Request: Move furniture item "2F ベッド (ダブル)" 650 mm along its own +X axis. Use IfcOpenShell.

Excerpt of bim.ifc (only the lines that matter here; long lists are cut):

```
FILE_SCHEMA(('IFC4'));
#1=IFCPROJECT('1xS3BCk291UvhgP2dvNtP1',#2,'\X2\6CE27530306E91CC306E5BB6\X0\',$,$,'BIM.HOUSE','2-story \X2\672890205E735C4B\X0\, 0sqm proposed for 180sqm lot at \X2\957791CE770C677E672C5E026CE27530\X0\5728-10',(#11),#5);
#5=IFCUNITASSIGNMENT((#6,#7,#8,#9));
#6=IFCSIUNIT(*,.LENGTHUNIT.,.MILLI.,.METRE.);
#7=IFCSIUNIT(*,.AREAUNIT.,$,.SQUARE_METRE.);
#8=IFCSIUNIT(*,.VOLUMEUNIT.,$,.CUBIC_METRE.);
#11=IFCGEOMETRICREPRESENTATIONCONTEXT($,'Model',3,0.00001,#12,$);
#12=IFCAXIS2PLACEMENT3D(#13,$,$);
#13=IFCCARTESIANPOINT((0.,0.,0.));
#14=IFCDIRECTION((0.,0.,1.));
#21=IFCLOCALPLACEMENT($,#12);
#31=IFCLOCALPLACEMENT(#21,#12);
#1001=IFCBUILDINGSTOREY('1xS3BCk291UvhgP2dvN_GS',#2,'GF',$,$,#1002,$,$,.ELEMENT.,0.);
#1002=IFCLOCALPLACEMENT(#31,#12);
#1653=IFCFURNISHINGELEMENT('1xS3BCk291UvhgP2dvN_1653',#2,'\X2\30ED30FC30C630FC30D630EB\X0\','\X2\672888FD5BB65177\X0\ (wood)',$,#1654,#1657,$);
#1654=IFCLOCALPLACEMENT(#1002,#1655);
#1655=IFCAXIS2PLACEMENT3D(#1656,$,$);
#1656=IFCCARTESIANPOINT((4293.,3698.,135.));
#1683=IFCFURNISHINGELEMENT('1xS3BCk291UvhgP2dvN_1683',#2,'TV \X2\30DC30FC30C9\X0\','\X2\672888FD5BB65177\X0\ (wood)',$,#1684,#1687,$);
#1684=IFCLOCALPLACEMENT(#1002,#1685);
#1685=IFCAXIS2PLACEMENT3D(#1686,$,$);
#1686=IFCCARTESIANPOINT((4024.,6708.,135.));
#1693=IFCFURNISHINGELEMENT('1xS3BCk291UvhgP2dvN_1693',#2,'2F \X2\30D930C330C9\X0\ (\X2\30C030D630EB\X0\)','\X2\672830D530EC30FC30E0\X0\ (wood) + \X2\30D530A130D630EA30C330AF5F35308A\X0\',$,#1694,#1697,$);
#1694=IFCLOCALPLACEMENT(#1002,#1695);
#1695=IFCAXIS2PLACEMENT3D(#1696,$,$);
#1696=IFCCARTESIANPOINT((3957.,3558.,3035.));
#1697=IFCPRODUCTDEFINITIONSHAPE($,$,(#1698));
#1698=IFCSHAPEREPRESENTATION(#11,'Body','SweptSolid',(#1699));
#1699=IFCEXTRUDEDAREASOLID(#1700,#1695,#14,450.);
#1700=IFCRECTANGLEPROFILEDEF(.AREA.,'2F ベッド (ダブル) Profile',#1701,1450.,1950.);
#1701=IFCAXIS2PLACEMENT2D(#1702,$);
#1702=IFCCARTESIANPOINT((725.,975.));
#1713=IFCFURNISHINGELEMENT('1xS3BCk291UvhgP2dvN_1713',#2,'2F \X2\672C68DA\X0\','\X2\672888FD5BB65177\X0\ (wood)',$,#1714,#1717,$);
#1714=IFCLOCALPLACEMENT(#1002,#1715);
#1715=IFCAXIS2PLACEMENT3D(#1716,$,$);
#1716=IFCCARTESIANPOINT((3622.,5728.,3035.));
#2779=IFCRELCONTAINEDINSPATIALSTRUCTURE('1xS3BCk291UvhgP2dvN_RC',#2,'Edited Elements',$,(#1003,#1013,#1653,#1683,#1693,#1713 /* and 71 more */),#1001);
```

```python
import ifcopenshell
import ifcopenshell.api.geometry
import ifcopenshell.util.placement

model = ifcopenshell.open("bim.ifc")

item = model.by_guid("1xS3BCk291UvhgP2dvN_1693")
matrix = ifcopenshell.util.placement.get_local_placement(item.ObjectPlacement)
matrix[:3, 3] += matrix[:3, 0] * 650.0
ifcopenshell.api.geometry.edit_object_placement(model, product=item, matrix=matrix, is_si=False)

print(ifcopenshell.util.placement.get_local_placement(item.ObjectPlacement).round(3) + 0.0)

model.write("bim-out.ifc")
```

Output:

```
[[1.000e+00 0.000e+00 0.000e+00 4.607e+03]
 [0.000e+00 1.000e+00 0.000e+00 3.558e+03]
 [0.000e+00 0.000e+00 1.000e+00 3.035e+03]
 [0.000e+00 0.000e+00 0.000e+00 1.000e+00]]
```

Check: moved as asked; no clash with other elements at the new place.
